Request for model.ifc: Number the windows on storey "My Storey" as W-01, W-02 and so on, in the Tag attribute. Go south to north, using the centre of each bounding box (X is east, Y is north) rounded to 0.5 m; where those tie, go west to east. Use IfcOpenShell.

First a look at what the model holds.

```python
import ifcopenshell
import ifcopenshell.util.element
import ifcopenshell.util.placement

model = ifcopenshell.open("model.ifc")
print(model.schema)
storey = next(s for s in model.by_type("IfcBuildingStorey") if s.Name == "My Storey")
windows = [e for e in ifcopenshell.util.element.get_decomposition(storey) if e.is_a("IfcWindow")]
for e in sorted(windows, key=lambda e: e.id()):
    origin = ifcopenshell.util.placement.get_local_placement(e.ObjectPlacement)[:3, 3]
    print(e.id(), e.Tag, e.Name, origin.round(2) + 0.0, sep=" | ")
```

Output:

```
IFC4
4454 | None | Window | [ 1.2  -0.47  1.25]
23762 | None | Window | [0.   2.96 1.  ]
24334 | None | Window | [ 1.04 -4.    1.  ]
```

```python
import ifcopenshell
import ifcopenshell.geom
import ifcopenshell.util.element
import ifcopenshell.util.shape

model = ifcopenshell.open("model.ifc")
settings = ifcopenshell.geom.settings()
settings.set("use-world-coords", True)


def centre(element):
    shape = ifcopenshell.geom.create_shape(settings, element)
    return ifcopenshell.util.shape.get_bbox_centroid(shape.geometry)


storey = next(s for s in model.by_type("IfcBuildingStorey") if s.Name == "My Storey")
windows = [e for e in ifcopenshell.util.element.get_decomposition(storey) if e.is_a("IfcWindow")]

# Insertion points can sit at a corner or the storey origin, so sort by the geometry (in metres).
centres = {e: centre(e) for e in windows}
windows.sort(key=lambda e: (round(centres[e][1] / 0.5), centres[e][0]))

for i, e in enumerate(windows, start=1):
    number = f"W-{i:02d}"
    e.Tag = number
    print(e.id(), number)

model.write("model_updated.ifc")
```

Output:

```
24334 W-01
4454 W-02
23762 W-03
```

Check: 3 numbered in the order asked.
